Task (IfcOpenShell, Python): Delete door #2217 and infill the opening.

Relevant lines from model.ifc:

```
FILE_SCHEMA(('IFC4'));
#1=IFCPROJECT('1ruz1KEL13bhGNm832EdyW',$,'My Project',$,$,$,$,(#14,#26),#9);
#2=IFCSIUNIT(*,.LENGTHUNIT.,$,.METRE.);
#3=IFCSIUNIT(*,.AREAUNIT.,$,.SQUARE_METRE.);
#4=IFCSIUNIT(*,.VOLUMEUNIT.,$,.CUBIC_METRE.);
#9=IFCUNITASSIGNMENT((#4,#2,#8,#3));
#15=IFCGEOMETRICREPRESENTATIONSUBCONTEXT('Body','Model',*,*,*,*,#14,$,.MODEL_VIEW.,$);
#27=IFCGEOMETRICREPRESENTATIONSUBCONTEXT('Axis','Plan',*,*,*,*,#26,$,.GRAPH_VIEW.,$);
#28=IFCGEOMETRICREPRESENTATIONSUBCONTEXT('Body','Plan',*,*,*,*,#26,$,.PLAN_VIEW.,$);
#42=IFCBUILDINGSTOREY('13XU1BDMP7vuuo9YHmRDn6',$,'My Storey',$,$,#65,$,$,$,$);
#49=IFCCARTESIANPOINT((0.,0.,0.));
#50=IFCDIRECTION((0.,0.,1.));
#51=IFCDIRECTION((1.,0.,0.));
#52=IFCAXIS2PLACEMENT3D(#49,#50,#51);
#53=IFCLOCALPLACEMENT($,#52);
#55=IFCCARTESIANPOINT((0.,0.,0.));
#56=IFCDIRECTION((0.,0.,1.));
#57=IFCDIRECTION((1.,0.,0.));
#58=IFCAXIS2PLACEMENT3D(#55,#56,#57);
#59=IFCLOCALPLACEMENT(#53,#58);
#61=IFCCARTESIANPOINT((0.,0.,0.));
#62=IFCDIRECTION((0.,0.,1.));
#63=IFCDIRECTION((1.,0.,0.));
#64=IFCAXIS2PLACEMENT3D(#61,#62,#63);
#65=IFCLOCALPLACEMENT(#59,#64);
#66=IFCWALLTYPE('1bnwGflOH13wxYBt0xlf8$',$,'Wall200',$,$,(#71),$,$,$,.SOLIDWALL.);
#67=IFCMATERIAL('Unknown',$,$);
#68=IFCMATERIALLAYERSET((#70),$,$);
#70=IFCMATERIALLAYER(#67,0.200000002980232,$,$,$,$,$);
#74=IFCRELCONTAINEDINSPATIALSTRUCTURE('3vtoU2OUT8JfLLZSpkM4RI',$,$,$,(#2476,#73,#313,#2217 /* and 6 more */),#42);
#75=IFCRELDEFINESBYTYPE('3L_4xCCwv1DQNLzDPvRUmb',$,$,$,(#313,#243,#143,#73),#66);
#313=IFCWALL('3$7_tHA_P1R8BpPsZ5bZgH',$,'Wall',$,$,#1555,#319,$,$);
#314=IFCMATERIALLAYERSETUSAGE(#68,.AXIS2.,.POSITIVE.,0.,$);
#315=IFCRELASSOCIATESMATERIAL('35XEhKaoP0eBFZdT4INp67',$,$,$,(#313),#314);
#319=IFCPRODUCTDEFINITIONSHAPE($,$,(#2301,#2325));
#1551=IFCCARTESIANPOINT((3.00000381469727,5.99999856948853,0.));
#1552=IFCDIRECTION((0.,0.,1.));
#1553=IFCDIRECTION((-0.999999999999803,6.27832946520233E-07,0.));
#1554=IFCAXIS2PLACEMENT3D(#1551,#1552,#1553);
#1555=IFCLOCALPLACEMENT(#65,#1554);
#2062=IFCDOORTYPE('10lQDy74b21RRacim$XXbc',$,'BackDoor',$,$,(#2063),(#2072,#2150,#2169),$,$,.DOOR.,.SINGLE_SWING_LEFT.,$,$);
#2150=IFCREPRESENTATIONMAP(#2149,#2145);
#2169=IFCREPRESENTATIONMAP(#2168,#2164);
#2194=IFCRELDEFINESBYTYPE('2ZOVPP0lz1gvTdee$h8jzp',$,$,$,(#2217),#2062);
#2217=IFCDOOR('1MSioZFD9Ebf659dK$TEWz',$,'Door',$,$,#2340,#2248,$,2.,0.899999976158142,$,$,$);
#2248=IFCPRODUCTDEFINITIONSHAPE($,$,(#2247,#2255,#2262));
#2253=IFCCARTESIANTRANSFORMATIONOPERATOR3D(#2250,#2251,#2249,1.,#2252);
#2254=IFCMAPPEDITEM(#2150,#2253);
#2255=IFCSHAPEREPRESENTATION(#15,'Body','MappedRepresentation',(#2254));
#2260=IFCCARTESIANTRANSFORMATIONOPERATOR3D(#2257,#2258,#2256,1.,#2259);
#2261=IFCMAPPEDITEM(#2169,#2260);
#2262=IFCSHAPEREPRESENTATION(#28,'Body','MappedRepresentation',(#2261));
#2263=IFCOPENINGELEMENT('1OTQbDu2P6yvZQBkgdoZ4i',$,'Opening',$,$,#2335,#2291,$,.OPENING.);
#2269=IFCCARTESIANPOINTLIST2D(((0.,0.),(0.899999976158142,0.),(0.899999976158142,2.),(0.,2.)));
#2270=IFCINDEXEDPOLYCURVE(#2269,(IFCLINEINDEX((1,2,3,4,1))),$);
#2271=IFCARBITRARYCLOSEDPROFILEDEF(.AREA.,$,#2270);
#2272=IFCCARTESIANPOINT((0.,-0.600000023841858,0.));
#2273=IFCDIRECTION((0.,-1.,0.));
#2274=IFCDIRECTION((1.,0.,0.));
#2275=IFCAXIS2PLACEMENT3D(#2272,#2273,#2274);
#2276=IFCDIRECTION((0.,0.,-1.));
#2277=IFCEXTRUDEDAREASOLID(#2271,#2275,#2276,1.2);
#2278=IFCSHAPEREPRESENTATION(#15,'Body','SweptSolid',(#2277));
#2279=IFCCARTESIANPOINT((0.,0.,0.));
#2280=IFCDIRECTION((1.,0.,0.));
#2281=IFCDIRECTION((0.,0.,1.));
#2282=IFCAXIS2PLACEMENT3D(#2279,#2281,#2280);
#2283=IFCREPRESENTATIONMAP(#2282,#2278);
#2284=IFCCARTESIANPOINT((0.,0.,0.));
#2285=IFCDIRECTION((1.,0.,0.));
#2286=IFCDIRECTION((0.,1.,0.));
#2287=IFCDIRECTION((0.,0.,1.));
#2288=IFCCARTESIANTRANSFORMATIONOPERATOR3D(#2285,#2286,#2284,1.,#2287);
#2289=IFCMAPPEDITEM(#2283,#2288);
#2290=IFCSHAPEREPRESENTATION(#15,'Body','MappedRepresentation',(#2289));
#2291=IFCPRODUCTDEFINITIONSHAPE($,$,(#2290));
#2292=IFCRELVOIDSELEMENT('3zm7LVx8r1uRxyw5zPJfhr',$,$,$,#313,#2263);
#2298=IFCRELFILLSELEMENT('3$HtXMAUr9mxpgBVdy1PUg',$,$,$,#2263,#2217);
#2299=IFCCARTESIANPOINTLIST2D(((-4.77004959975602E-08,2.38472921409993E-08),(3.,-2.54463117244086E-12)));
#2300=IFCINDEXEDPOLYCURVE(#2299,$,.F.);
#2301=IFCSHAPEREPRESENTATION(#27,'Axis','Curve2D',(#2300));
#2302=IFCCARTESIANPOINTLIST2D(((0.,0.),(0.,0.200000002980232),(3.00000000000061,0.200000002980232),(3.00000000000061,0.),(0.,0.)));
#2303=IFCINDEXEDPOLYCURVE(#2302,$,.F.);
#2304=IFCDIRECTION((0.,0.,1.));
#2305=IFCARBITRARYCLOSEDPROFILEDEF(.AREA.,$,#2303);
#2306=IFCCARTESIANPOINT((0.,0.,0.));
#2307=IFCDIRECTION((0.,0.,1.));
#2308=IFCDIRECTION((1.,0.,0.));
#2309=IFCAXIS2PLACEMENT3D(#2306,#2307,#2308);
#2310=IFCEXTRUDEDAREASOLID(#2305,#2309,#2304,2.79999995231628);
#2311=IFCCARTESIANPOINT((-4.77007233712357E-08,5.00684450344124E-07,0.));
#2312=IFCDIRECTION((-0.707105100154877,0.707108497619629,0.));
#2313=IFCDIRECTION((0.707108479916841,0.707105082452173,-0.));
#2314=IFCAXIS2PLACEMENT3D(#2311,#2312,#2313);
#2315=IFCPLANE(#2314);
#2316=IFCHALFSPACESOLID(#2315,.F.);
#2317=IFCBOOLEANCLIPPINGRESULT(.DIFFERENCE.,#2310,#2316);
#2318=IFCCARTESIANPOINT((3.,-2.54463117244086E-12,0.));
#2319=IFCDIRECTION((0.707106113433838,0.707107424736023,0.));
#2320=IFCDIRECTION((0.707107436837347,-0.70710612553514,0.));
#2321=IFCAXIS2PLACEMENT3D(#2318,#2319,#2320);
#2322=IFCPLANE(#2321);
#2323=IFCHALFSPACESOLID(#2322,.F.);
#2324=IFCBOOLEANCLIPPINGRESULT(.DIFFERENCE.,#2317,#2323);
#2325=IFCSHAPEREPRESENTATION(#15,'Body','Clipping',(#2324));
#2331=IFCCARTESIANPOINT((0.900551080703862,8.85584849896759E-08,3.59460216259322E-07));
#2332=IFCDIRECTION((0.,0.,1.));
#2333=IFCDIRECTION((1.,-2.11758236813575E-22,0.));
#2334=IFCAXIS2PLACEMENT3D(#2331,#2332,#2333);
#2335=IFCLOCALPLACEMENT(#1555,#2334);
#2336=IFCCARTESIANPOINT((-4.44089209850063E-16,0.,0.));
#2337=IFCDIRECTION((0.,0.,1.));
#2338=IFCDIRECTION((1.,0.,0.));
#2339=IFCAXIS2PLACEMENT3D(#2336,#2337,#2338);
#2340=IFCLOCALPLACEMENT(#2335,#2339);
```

```python
import ifcopenshell
import ifcopenshell.api.feature
import ifcopenshell.api.root
import ifcopenshell.geom
import ifcopenshell.util.shape

model = ifcopenshell.open("model.ifc")
settings = ifcopenshell.geom.settings()


def volume(element):
    """Net volume in cubic metres, openings subtracted."""
    shape = ifcopenshell.geom.create_shape(settings, element)
    return ifcopenshell.util.shape.get_volume(shape.geometry)


door = model.by_id(2217)
opening = door.FillsVoids[0].RelatingOpeningElement
wall = opening.VoidsElements[0].RelatingBuildingElement
before = volume(wall)

ifcopenshell.api.root.remove_product(model, product=door)
ifcopenshell.api.feature.remove_feature(model, feature=opening)

after = volume(wall)

print(f"wall volume {before:.3f} -> {after:.3f} m3")

model.write("model_rev.ifc")
```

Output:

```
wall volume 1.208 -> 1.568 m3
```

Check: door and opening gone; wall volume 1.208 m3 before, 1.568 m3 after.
